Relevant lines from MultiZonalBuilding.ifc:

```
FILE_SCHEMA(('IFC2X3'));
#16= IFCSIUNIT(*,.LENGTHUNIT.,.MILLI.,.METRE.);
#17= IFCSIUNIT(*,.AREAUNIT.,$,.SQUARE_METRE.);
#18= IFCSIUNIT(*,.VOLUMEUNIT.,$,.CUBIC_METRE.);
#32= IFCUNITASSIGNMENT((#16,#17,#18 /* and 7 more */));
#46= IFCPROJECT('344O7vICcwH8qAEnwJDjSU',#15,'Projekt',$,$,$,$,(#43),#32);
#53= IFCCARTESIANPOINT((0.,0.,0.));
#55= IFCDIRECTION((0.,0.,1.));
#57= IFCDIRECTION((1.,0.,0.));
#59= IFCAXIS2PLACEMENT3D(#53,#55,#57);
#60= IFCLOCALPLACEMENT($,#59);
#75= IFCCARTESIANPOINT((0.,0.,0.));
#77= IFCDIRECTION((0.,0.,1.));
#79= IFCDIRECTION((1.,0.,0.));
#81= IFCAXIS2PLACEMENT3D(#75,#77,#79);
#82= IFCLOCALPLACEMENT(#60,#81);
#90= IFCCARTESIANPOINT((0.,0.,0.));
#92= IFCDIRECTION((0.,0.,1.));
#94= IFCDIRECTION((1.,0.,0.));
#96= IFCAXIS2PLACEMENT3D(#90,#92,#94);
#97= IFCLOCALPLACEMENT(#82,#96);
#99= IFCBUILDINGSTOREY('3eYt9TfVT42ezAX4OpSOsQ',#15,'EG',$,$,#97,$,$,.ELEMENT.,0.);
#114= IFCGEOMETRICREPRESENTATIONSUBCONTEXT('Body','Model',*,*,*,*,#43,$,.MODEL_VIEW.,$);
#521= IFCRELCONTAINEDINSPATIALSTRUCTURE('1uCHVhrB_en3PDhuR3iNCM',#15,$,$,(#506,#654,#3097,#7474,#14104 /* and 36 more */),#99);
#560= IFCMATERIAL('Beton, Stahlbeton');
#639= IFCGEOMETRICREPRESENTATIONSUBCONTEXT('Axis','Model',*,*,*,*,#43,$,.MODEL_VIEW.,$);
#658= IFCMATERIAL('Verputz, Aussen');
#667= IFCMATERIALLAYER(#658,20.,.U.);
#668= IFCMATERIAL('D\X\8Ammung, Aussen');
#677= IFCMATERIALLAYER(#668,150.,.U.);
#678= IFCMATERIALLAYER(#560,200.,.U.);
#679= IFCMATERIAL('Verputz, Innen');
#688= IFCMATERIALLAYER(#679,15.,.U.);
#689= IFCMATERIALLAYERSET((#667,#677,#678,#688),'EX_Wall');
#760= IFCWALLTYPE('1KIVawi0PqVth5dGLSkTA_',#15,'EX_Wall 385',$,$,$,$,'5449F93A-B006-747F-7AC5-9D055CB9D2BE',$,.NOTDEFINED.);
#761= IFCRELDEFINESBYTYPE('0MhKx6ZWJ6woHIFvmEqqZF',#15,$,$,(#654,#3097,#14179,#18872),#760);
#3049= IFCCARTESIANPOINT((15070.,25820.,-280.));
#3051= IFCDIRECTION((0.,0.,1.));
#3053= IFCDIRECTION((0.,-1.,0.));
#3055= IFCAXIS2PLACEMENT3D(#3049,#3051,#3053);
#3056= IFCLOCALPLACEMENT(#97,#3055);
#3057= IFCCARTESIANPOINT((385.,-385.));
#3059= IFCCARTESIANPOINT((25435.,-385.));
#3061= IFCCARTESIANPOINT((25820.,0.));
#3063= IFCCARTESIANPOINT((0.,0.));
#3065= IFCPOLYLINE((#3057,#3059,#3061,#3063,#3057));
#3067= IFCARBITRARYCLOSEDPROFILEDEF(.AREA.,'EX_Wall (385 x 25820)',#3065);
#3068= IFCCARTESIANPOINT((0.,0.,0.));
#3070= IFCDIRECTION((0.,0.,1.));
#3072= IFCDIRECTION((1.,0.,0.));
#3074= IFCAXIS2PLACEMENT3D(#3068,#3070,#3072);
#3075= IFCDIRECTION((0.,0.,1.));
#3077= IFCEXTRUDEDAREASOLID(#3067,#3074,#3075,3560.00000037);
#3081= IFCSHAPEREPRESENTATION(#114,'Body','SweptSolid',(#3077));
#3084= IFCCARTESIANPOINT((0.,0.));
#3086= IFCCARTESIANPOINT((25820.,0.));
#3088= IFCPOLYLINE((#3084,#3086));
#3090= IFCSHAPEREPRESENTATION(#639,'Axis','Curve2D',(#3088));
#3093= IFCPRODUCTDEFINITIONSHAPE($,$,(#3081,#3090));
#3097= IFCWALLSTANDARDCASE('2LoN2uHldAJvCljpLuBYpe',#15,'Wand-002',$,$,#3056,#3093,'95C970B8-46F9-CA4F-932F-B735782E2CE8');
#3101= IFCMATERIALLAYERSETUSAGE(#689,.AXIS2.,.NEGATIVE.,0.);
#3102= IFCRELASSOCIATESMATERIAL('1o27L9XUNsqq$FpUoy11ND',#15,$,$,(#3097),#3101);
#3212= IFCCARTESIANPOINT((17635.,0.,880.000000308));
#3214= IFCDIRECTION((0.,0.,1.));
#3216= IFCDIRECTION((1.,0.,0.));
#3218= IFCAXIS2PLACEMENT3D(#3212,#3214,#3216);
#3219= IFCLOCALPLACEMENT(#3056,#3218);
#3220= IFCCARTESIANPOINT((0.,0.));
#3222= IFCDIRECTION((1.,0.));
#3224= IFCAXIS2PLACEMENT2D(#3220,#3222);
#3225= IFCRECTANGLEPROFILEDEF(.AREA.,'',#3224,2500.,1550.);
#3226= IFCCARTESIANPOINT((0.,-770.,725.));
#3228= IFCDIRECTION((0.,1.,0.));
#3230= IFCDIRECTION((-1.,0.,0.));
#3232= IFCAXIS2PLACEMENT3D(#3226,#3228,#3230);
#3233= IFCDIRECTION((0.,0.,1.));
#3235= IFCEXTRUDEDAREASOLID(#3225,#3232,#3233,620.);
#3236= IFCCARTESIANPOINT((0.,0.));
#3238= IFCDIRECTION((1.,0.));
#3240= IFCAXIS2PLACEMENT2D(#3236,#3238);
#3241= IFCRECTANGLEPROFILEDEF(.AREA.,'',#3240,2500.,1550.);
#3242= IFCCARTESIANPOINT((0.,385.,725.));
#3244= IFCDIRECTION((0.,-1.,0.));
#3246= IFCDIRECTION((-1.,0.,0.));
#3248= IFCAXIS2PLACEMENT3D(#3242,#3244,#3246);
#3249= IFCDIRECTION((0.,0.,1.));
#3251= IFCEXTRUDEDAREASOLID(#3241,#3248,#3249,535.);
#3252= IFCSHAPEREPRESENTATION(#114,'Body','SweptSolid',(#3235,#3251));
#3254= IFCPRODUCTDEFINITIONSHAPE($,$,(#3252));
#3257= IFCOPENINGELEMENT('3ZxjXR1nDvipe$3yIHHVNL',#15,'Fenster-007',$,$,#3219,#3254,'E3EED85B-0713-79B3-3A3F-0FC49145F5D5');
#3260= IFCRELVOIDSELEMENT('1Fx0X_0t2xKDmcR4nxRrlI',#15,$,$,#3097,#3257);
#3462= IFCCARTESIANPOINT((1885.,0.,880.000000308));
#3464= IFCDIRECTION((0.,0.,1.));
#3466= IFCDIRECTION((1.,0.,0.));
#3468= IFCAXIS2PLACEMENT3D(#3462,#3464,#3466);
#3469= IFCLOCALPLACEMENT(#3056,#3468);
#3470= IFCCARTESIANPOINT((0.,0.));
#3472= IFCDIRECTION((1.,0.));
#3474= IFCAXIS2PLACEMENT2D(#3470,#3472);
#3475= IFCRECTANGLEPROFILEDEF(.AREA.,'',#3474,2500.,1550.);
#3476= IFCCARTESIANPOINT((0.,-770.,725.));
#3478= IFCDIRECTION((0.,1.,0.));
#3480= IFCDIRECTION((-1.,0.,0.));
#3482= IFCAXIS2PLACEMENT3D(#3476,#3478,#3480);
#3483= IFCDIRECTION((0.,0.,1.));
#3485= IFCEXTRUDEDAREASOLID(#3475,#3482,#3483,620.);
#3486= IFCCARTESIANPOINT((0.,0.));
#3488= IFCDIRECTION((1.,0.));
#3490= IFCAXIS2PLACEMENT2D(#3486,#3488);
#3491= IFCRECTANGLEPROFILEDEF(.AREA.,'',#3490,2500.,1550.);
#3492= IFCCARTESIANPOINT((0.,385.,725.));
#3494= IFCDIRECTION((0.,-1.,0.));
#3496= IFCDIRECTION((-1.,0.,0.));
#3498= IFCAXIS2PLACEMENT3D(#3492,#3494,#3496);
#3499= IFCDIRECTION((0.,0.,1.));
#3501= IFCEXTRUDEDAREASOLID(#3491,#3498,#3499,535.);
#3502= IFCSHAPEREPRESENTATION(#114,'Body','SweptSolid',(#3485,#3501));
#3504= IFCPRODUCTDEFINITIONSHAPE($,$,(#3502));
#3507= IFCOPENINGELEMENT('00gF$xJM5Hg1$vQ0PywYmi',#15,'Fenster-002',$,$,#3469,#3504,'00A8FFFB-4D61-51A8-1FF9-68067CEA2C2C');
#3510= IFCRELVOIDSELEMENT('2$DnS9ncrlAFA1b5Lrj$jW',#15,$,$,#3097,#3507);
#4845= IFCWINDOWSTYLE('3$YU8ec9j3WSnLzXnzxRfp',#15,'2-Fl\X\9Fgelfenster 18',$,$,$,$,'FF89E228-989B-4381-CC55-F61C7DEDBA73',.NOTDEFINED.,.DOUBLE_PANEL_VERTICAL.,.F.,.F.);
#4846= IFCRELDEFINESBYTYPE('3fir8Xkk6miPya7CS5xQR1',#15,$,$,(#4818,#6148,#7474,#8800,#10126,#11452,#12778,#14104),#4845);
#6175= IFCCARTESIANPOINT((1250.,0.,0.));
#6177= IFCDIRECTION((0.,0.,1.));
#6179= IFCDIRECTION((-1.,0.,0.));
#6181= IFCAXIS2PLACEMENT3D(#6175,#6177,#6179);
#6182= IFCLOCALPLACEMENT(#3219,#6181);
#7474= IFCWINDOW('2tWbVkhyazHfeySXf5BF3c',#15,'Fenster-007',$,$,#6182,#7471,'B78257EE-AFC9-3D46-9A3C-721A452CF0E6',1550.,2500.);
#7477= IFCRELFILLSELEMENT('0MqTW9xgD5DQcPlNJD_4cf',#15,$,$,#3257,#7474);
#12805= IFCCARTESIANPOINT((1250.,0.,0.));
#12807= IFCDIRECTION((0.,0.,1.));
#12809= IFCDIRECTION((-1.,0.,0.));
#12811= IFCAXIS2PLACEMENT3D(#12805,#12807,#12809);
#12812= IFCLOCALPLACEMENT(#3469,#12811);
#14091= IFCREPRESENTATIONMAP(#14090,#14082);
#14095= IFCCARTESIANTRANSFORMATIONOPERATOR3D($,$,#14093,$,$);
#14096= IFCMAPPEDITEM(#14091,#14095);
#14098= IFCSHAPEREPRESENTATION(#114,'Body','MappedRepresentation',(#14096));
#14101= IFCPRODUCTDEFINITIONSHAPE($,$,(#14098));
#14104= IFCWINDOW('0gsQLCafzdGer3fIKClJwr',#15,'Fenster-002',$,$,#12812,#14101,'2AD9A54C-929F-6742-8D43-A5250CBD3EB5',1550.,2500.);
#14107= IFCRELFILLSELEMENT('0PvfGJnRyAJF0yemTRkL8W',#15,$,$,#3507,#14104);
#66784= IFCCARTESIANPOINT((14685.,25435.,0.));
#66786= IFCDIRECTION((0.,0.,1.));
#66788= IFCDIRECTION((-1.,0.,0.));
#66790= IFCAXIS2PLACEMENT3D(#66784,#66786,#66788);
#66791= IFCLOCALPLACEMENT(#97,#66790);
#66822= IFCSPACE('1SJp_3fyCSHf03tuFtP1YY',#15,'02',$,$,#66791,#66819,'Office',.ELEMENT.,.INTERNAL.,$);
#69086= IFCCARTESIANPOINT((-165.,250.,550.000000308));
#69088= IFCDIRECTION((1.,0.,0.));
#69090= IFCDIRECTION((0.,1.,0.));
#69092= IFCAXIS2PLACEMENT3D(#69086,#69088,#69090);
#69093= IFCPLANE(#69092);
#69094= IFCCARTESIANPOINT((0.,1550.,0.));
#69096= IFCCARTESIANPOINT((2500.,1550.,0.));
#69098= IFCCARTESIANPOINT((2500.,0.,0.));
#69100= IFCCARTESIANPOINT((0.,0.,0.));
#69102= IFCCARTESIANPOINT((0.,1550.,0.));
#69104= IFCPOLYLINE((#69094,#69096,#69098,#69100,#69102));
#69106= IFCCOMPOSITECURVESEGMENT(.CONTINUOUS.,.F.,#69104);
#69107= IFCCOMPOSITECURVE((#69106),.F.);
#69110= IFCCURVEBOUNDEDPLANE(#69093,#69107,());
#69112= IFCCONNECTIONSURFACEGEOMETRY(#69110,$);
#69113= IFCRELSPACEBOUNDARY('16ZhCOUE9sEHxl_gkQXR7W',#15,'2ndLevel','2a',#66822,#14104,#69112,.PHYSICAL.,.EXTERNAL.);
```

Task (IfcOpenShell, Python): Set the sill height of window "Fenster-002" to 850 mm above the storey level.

```python
import numpy as np
import ifcopenshell
import ifcopenshell.api.geometry
import ifcopenshell.geom
import ifcopenshell.util.element
import ifcopenshell.util.placement
import ifcopenshell.util.shape
import ifcopenshell.util.unit

model = ifcopenshell.open("MultiZonalBuilding.ifc")
unit_scale = ifcopenshell.util.unit.calculate_unit_scale(model)

window = model.by_guid("0gsQLCafzdGer3fIKClJwr")
opening = window.FillsVoids[0].RelatingOpeningElement
storey = ifcopenshell.util.element.get_container(window, ifc_class="IfcBuildingStorey")
level = ifcopenshell.util.placement.get_local_placement(storey.ObjectPlacement)[2, 3]

# The opening's origin need not be at the sill, so measure its lowest point.
shape = ifcopenshell.geom.create_shape(ifcopenshell.geom.settings(), opening)
bottom = ifcopenshell.util.shape.get_shape_bottom_elevation(shape, shape.geometry) / unit_scale
dz = level + 0.85 / unit_scale - bottom

shift = np.array([0.0, 0.0, dz])
# The window is placed relative to its opening, so it follows when the opening moves.
matrix = ifcopenshell.util.placement.get_local_placement(opening.ObjectPlacement)
matrix[:3, 3] += shift
ifcopenshell.api.geometry.edit_object_placement(
    model, product=opening, matrix=matrix, is_si=False, should_transform_children=True
)

# Space boundary surfaces are stored in each space's coordinates; move them too.
for rel in window.ProvidesBoundaries:
    if not rel.ConnectionGeometry:
        continue
    surface = rel.ConnectionGeometry.SurfaceOnRelatingElement.BasisSurface
    space_matrix = ifcopenshell.util.placement.get_local_placement(rel.RelatingSpace.ObjectPlacement)
    point = np.array(surface.Position.Location.Coordinates) + space_matrix[:3, :3].T @ shift
    surface.Position = model.createIfcAxis2Placement3D(
        model.createIfcCartesianPoint(point.tolist()), surface.Position.Axis, surface.Position.RefDirection
    )

print(f"moved by {dz * unit_scale:+.3f} m")

model.write("MultiZonalBuilding-out.ifc")
```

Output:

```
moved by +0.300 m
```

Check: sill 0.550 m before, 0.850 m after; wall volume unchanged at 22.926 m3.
